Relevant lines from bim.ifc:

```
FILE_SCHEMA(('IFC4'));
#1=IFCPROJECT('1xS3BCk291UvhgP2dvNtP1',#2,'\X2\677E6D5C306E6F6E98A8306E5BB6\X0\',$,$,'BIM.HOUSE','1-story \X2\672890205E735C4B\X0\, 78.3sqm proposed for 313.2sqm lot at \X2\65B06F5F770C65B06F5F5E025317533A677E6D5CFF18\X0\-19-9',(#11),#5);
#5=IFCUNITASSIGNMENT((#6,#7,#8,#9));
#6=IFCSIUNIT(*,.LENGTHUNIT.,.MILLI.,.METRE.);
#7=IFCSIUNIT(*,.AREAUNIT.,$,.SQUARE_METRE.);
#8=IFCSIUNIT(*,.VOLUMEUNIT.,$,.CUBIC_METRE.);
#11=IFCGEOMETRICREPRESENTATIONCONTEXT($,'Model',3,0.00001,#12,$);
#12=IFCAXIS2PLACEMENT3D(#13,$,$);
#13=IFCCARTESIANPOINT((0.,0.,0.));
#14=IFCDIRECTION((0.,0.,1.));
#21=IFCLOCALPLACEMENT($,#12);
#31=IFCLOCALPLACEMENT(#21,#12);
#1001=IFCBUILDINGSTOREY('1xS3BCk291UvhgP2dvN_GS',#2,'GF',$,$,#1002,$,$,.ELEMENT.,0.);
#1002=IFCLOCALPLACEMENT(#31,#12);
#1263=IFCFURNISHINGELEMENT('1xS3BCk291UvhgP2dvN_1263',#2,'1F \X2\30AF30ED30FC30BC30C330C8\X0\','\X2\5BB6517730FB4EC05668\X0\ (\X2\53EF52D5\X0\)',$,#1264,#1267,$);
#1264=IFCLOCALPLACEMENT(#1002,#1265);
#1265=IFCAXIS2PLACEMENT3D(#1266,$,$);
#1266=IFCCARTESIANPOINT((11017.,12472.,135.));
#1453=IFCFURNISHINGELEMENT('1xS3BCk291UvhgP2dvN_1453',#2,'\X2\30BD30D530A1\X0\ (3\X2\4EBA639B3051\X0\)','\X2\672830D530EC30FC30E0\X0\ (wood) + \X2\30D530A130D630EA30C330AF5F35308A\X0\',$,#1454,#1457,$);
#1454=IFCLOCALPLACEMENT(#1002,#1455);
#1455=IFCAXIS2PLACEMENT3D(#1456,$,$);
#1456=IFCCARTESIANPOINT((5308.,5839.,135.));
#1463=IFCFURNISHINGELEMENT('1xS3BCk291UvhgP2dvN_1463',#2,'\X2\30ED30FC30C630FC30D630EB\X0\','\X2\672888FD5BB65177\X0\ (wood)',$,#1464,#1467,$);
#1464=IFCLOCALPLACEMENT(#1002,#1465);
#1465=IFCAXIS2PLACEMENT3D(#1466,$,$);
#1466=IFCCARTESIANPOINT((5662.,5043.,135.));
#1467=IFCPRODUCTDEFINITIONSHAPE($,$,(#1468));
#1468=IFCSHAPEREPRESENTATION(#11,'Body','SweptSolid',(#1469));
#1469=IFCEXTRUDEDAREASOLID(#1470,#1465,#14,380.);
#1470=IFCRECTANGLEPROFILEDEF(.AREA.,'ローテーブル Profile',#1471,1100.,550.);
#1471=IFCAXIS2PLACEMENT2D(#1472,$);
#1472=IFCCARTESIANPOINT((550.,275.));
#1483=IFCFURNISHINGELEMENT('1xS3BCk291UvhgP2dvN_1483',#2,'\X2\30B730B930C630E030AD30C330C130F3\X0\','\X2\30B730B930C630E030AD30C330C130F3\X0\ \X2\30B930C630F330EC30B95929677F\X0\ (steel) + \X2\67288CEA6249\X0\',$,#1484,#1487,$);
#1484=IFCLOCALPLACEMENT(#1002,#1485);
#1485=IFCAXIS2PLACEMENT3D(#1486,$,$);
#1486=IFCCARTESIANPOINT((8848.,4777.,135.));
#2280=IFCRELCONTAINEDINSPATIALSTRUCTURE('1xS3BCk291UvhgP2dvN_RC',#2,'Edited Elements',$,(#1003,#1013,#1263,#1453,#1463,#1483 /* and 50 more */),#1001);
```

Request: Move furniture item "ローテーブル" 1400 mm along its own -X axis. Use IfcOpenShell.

```python
import ifcopenshell
import ifcopenshell.api.geometry
import ifcopenshell.util.placement
import ifcopenshell.util.unit

model = ifcopenshell.open("bim.ifc")
unit_scale = ifcopenshell.util.unit.calculate_unit_scale(model)

item = model.by_guid("1xS3BCk291UvhgP2dvN_1463")
matrix = ifcopenshell.util.placement.get_local_placement(item.ObjectPlacement)
matrix[:3, 3] -= matrix[:3, 0] * 1.4 / unit_scale
ifcopenshell.api.geometry.edit_object_placement(model, product=item, matrix=matrix, is_si=False)

print(ifcopenshell.util.placement.get_local_placement(item.ObjectPlacement).round(3) + 0.0)

model.write("bim_rev.ifc")
```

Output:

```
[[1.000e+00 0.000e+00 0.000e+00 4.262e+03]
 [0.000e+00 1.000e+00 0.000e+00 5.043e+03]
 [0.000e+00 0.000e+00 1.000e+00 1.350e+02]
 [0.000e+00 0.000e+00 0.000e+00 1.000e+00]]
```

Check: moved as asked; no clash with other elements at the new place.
